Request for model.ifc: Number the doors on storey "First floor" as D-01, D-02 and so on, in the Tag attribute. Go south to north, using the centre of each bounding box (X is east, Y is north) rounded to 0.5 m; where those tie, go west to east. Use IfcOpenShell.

First a look at what the model holds.

```python
import ifcopenshell
import ifcopenshell.util.element
import ifcopenshell.util.placement

model = ifcopenshell.open("model.ifc")
print(model.schema)
storey = next(s for s in model.by_type("IfcBuildingStorey") if s.Name == "First floor")
doors = [e for e in ifcopenshell.util.element.get_decomposition(storey) if e.is_a("IfcDoor")]
for e in sorted(doors, key=lambda e: e.id()):
    origin = ifcopenshell.util.placement.get_local_placement(e.ObjectPlacement)[:3, 3]
    print(e.id(), e.Tag, e.Name, origin.round(2) + 0.0, sep=" | ")
```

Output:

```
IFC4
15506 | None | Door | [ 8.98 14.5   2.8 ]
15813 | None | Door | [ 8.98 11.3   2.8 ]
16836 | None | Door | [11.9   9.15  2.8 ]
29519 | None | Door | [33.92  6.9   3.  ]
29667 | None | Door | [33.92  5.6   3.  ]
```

```python
import ifcopenshell
import ifcopenshell.geom
import ifcopenshell.util.element
import ifcopenshell.util.shape

model = ifcopenshell.open("model.ifc")
settings = ifcopenshell.geom.settings()
settings.set("use-world-coords", True)


def centre(element):
    shape = ifcopenshell.geom.create_shape(settings, element)
    return ifcopenshell.util.shape.get_bbox_centroid(shape.geometry)


storey = next(s for s in model.by_type("IfcBuildingStorey") if s.Name == "First floor")
doors = [e for e in ifcopenshell.util.element.get_decomposition(storey) if e.is_a("IfcDoor")]

# Insertion points can sit at a corner or the storey origin, so sort by the geometry (in metres).
centres = {e: centre(e) for e in doors}
doors.sort(key=lambda e: (round(centres[e][1] / 0.5), centres[e][0]))

for i, e in enumerate(doors, start=1):
    number = f"D-{i:02d}"
    e.Tag = number
    print(e.id(), number)

model.write("model-out.ifc")
```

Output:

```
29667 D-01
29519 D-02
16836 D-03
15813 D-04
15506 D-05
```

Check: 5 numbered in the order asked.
